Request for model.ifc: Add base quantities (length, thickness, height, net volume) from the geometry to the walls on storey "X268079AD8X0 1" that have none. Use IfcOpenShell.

First a look at what the model holds.

```python
import ifcopenshell
import ifcopenshell.util.element
import ifcopenshell.util.unit

model = ifcopenshell.open("model.ifc")
print(model.schema)
for unit_type in ("LENGTHUNIT", "AREAUNIT", "VOLUMEUNIT"):
    print(unit_type, ifcopenshell.util.unit.calculate_unit_scale(model, unit_type))
storey = next(s for s in model.by_type("IfcBuildingStorey") if s.Name == "X268079AD8X0 1")
walls = [e for e in ifcopenshell.util.element.get_decomposition(storey) if e.is_a("IfcWall")]
for e in sorted(walls, key=lambda e: e.id()):
    print(e.id(), e.is_a(), e.Name, list(ifcopenshell.util.element.get_psets(e, qtos_only=True)), sep=" | ")
```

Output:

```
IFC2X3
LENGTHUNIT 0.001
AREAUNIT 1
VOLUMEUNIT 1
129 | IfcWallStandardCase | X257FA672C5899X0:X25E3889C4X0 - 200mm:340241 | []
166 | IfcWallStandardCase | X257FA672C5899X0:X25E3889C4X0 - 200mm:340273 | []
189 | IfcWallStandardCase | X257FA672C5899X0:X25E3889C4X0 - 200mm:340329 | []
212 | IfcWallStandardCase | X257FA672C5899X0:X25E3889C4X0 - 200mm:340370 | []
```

```python
import ifcopenshell
import ifcopenshell.api.pset
import ifcopenshell.geom
import ifcopenshell.util.element
import ifcopenshell.util.shape
import ifcopenshell.util.unit

model = ifcopenshell.open("model.ifc")
unit_scale = ifcopenshell.util.unit.calculate_unit_scale(model)
volume_scale = ifcopenshell.util.unit.calculate_unit_scale(model, "VOLUMEUNIT")
settings = ifcopenshell.geom.settings()

storey = next(s for s in model.by_type("IfcBuildingStorey") if s.Name == "X268079AD8X0 1")
walls = [e for e in ifcopenshell.util.element.get_decomposition(storey) if e.is_a("IfcWall")]

for e in sorted(walls, key=lambda e: e.id()):
    if ifcopenshell.util.element.get_psets(e, qtos_only=True, should_inherit=False):
        continue
    # Geometry comes back in metres, in the element's own axes.
    shape = ifcopenshell.geom.create_shape(settings, e)
    values = {
        "Length": ifcopenshell.util.shape.get_x(shape.geometry) / unit_scale,
        "Width": ifcopenshell.util.shape.get_y(shape.geometry) / unit_scale,
        "Height": ifcopenshell.util.shape.get_z(shape.geometry) / unit_scale,
        "NetVolume": ifcopenshell.util.shape.get_volume(shape.geometry) / volume_scale,
    }
    qto = ifcopenshell.api.pset.add_qto(model, product=e, name="BaseQuantities")
    ifcopenshell.api.pset.edit_qto(model, qto=qto, properties=values)
    print(e.id(), {k: round(v, 3) for k, v in values.items()})

model.write("model_rev.ifc")
```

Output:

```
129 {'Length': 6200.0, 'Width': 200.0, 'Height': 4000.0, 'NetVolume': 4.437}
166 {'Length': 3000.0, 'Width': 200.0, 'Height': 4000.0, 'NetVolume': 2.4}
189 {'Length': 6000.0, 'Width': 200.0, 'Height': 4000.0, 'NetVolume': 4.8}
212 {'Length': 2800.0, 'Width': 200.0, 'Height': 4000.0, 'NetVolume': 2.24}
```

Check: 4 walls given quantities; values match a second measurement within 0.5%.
